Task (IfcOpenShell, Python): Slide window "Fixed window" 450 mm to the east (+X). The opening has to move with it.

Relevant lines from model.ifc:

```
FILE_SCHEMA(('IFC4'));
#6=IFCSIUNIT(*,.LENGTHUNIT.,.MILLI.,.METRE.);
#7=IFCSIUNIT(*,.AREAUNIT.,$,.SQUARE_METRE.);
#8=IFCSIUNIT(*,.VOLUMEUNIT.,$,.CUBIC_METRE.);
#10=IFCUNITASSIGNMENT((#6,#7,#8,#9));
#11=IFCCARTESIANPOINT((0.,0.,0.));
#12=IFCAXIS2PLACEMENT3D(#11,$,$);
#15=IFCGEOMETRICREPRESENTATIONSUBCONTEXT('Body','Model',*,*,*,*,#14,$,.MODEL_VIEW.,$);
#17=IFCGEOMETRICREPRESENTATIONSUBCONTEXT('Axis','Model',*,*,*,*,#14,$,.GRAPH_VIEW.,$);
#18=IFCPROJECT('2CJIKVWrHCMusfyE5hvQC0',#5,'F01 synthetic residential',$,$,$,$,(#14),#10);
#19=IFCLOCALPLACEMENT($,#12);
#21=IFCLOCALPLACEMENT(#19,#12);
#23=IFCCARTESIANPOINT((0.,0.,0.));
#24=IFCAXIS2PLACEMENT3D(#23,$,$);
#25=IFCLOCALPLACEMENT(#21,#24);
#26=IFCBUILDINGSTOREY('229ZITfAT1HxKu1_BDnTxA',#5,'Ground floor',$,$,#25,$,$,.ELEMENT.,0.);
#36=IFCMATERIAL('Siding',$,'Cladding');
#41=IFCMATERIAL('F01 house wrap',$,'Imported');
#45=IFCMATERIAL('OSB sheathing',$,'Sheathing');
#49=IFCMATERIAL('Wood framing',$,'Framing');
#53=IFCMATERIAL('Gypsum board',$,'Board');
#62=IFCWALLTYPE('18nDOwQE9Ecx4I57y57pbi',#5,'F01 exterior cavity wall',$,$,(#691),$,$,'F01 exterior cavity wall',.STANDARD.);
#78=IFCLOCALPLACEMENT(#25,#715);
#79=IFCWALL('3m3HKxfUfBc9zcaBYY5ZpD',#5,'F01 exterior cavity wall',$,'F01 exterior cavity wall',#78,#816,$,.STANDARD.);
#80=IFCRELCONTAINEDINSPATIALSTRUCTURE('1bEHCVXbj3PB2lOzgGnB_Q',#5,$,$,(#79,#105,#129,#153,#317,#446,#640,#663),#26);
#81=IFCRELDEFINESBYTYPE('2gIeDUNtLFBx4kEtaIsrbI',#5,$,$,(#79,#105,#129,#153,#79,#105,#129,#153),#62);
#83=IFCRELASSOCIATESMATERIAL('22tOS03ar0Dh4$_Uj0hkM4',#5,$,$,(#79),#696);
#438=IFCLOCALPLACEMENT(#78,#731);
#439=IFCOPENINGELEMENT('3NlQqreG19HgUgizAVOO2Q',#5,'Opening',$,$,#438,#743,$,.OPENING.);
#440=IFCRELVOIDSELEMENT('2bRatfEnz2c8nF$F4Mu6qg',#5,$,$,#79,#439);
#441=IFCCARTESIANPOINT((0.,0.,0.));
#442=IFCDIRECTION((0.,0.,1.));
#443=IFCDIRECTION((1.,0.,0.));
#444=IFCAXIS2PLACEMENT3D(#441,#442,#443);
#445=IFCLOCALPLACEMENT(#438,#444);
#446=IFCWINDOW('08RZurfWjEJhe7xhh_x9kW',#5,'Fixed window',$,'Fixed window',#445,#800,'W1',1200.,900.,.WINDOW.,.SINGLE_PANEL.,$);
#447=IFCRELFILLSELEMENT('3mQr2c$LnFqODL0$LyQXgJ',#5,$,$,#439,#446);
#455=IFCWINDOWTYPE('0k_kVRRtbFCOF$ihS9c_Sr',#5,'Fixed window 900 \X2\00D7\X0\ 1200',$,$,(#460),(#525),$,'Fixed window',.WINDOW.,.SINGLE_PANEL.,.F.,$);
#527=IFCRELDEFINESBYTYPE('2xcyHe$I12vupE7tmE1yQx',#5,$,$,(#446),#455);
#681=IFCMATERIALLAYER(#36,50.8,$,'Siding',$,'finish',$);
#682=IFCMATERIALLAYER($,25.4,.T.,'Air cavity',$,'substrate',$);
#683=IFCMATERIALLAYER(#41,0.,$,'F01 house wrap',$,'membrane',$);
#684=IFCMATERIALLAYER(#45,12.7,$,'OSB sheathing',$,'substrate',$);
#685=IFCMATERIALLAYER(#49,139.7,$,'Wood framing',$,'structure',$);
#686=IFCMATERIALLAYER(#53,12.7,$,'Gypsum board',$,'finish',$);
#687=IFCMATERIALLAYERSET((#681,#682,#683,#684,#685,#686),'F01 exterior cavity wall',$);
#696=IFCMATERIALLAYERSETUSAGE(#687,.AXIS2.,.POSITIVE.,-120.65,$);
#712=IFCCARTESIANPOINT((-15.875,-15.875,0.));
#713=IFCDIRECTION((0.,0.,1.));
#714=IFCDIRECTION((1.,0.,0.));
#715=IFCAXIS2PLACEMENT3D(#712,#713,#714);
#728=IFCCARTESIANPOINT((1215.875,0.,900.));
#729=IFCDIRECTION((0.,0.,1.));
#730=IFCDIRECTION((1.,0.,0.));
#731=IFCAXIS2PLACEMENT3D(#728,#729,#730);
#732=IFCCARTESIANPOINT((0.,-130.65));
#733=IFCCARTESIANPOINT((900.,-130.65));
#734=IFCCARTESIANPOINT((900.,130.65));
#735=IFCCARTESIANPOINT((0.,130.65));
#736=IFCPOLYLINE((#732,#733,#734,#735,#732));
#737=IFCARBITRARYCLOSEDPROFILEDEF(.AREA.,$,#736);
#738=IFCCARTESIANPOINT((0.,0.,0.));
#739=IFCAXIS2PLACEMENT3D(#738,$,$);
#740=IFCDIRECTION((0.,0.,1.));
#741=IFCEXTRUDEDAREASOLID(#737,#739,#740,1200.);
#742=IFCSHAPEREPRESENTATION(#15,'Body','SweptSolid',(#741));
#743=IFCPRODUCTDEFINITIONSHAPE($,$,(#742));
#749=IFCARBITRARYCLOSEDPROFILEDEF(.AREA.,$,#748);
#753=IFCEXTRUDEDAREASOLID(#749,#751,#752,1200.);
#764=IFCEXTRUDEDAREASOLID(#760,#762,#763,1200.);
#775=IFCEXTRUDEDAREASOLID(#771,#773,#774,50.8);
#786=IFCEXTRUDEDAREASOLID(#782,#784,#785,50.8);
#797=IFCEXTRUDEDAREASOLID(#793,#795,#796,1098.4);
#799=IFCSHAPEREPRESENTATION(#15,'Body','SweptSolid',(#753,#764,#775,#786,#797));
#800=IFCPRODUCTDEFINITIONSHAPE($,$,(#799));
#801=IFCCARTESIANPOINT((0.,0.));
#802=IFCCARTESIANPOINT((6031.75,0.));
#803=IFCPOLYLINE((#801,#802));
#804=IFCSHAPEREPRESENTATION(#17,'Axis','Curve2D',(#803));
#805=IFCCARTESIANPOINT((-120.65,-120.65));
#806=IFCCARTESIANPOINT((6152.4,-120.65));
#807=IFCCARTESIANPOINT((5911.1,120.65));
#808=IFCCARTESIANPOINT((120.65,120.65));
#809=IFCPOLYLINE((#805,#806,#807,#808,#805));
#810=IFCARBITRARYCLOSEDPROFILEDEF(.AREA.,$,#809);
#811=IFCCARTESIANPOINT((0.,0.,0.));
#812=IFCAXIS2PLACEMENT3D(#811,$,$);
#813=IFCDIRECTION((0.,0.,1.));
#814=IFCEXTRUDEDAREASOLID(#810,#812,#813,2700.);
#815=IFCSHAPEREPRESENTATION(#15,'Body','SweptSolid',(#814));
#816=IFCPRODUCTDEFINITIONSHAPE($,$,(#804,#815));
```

```python
import ifcopenshell
import ifcopenshell.api.geometry
import ifcopenshell.util.placement

model = ifcopenshell.open("model.ifc")

window = model.by_guid("08RZurfWjEJhe7xhh_x9kW")
opening = window.FillsVoids[0].RelatingOpeningElement
wall = opening.VoidsElements[0].RelatingBuildingElement

wall_matrix = ifcopenshell.util.placement.get_local_placement(wall.ObjectPlacement)
shift = wall_matrix[:3, 0] * 450.0
before = ifcopenshell.util.placement.get_local_placement(window.ObjectPlacement)[:3, 3].copy()

# The window is placed relative to its opening, so it follows when the opening moves.
matrix = ifcopenshell.util.placement.get_local_placement(opening.ObjectPlacement)
matrix[:3, 3] += shift
ifcopenshell.api.geometry.edit_object_placement(
    model, product=opening, matrix=matrix, is_si=False, should_transform_children=True
)

after = ifcopenshell.util.placement.get_local_placement(window.ObjectPlacement)[:3, 3]
print("window moved by", (after - before).round(3) + 0.0)

model.write("model_v2.ifc")
```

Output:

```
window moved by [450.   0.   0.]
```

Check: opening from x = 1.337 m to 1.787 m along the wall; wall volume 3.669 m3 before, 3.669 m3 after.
